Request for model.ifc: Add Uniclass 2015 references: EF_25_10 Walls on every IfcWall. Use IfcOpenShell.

First a look at what the model holds.

```python
import ifcopenshell

model = ifcopenshell.open("model.ifc")
print(model.schema)
print("classifications:", [c.Name for c in model.by_type("IfcClassification")])
for ifc_class in ("IfcDoor", "IfcRoof", "IfcStair", "IfcWall", "IfcWindow"):
    print(ifc_class, len(model.by_type(ifc_class)))
```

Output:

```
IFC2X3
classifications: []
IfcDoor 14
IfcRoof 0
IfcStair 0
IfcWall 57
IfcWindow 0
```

```python
import ifcopenshell
import ifcopenshell.api.classification

model = ifcopenshell.open("model.ifc")

# IFC2X3 requires Source and Edition and has no link from the project to the system.
system = model.create_entity("IfcClassification", Source="NBS", Edition="2015", Name="Uniclass 2015")

codes = {
    "IfcWall": ("EF_25_10", "Walls"),
}
for ifc_class, (code, name) in codes.items():
    products = model.by_type(ifc_class)
    ifcopenshell.api.classification.add_reference(
        model, products=products, classification=system, identification=code, name=name
    )
    print(code, len(products))

model.write("model_rev.ifc")
```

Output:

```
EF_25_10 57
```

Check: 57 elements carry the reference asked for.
